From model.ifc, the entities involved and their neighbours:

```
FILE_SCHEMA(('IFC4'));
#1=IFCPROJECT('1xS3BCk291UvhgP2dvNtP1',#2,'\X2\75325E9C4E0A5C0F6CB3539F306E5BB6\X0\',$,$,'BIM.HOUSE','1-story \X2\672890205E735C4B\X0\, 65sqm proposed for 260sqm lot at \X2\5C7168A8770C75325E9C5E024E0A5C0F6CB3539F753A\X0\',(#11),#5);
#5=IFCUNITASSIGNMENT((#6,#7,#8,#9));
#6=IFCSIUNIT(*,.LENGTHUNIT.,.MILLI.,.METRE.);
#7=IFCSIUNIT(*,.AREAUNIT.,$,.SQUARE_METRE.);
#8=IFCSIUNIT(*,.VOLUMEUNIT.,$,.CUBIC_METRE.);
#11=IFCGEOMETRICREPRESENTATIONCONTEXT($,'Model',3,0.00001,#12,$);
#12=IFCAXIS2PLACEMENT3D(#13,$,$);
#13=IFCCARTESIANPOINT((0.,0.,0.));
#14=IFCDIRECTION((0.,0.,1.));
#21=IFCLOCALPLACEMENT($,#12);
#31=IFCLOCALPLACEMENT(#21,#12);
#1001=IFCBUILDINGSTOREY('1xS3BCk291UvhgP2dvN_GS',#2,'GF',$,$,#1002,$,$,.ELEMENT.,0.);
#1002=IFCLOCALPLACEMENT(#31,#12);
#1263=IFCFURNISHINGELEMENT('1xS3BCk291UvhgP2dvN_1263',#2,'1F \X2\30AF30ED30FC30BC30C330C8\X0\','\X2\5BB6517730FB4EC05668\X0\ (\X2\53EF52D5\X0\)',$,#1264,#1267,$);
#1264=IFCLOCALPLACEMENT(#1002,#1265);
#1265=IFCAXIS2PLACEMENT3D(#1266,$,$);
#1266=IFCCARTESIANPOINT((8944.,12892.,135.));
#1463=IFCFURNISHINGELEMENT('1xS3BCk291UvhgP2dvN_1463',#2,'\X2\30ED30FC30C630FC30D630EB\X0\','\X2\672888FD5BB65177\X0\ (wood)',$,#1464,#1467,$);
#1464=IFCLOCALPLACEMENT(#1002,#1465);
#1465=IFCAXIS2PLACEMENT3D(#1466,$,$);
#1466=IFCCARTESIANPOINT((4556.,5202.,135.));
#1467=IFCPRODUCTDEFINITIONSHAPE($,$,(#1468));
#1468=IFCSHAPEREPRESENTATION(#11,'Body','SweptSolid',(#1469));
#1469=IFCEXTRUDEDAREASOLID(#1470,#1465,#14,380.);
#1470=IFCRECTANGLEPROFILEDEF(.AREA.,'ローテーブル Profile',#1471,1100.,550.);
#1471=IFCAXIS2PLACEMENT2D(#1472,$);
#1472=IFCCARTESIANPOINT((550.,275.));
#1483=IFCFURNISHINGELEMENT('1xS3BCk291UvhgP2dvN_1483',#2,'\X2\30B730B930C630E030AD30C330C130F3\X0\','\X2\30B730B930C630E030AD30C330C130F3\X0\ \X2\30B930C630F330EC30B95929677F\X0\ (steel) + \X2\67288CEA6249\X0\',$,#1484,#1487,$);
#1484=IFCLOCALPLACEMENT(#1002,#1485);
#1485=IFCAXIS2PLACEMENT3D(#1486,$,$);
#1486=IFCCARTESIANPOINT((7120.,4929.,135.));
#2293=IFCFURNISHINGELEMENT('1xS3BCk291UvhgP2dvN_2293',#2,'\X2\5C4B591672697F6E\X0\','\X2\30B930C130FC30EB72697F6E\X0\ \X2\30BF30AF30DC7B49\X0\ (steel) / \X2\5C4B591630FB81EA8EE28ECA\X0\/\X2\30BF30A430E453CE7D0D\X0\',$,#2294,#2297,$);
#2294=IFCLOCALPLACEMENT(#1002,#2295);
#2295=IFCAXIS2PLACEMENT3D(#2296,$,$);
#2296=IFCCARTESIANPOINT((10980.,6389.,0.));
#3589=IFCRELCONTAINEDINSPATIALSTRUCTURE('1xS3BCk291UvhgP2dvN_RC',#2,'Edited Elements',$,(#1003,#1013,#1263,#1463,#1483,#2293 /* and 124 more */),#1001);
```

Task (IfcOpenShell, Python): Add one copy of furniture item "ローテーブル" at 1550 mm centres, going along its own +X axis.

```python
import ifcopenshell
import ifcopenshell.api.geometry
import ifcopenshell.api.root
import ifcopenshell.util.element
import ifcopenshell.util.placement

model = ifcopenshell.open("model.ifc")


def reuse_history(source, copy):
    """copy_class also copies each property set's owner history, people and application; keep the originals."""
    for rel in copy.IsDefinedBy:
        if rel.is_a("IfcRelDefinesByProperties") and (history := rel.RelatingPropertyDefinition.OwnerHistory):
            rel.RelatingPropertyDefinition.OwnerHistory = source.OwnerHistory
            ifcopenshell.util.element.remove_deep2(model, history)


source = model.by_guid("1xS3BCk291UvhgP2dvN_1463")
base = ifcopenshell.util.placement.get_local_placement(source.ObjectPlacement)
step = base[:3, 0] * 1550.0

for i in range(1, 2):
    copy = ifcopenshell.api.root.copy_class(model, product=source)
    copy.Representation = ifcopenshell.util.element.copy_deep(
        model, source.Representation, exclude=["IfcGeometricRepresentationContext", "IfcRepresentationMap"]
    )
    reuse_history(source, copy)
    matrix = base.copy()
    matrix[:3, 3] += i * step
    print("added at", matrix[:3, 3].round(3) + 0.0)
    ifcopenshell.api.geometry.edit_object_placement(model, product=copy, matrix=matrix, is_si=False)

model.write("model-out.ifc")
```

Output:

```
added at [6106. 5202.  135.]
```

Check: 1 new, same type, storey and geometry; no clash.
